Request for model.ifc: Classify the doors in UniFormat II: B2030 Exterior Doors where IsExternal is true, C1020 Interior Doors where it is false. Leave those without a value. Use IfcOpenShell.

First a look at what the model holds.

```python
import ifcopenshell
import ifcopenshell.util.element

model = ifcopenshell.open("model.ifc")
print(model.schema)
print("classifications:", [c.Name for c in model.by_type("IfcClassification")])
values = [ifcopenshell.util.element.get_pset(e, "Pset_DoorCommon", "IsExternal") for e in model.by_type("IfcDoor")]
for value in (True, False, None):
    print("IsExternal", value, values.count(value))
```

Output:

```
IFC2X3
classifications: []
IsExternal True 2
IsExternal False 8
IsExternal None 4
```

```python
import ifcopenshell
import ifcopenshell.api.classification
import ifcopenshell.util.element

model = ifcopenshell.open("model.ifc")

# IFC2X3 requires Source and Edition and has no link from the project to the system.
system = model.create_entity("IfcClassification", Source="ASTM", Edition="E1557", Name="UniFormat II")

doors = model.by_type("IfcDoor")
external = {e: ifcopenshell.util.element.get_pset(e, "Pset_DoorCommon", "IsExternal") for e in doors}
for flag, code, name in ((True, "B2030", "Exterior Doors"), (False, "C1020", "Interior Doors")):
    products = [e for e in doors if external[e] is flag]
    ifcopenshell.api.classification.add_reference(
        model, products=products, classification=system, identification=code, name=name
    )
    print(code, len(products))

model.write("model_rev.ifc")
```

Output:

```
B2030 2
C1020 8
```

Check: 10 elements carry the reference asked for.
